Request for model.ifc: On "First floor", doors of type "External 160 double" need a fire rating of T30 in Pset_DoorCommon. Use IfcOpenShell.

First a look at what the model holds.

```python
import ifcopenshell
import ifcopenshell.util.element

model = ifcopenshell.open("model.ifc")
print(model.schema)
storey = next(s for s in model.by_type("IfcBuildingStorey") if s.Name == "First floor")
doors = [e for e in ifcopenshell.util.element.get_decomposition(storey) if e.is_a("IfcDoor")]
seen = {}
for e in doors:
    element_type = ifcopenshell.util.element.get_type(e)
    key = (element_type.Name if element_type != e and element_type else None, ifcopenshell.util.element.get_pset(e, "Pset_DoorCommon", "FireRating"))
    seen[key] = seen.get(key, 0) + 1
for (name, value), count in sorted(seen.items(), key=str):
    print(count, "x", name, "|", value)
```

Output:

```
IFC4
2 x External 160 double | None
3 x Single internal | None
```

```python
import ifcopenshell
import ifcopenshell.api.pset
import ifcopenshell.util.element

model = ifcopenshell.open("model.ifc")

storey = next(s for s in model.by_type("IfcBuildingStorey") if s.Name == "First floor")
doors = [e for e in ifcopenshell.util.element.get_decomposition(storey) if e.is_a("IfcDoor")]

count = 0
for e in doors:
    element_type = ifcopenshell.util.element.get_type(e)
    if element_type in (None, e) or element_type.Name != "External 160 double":
        continue
    # add_pset returns the element's existing set when there is one.
    pset = ifcopenshell.api.pset.add_pset(model, product=e, name="Pset_DoorCommon")
    ifcopenshell.api.pset.edit_pset(model, pset=pset, properties={"FireRating": "T30"})
    count += 1

print(count, "doors updated")

model.write("model_edited.ifc")
```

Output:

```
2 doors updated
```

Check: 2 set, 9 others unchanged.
